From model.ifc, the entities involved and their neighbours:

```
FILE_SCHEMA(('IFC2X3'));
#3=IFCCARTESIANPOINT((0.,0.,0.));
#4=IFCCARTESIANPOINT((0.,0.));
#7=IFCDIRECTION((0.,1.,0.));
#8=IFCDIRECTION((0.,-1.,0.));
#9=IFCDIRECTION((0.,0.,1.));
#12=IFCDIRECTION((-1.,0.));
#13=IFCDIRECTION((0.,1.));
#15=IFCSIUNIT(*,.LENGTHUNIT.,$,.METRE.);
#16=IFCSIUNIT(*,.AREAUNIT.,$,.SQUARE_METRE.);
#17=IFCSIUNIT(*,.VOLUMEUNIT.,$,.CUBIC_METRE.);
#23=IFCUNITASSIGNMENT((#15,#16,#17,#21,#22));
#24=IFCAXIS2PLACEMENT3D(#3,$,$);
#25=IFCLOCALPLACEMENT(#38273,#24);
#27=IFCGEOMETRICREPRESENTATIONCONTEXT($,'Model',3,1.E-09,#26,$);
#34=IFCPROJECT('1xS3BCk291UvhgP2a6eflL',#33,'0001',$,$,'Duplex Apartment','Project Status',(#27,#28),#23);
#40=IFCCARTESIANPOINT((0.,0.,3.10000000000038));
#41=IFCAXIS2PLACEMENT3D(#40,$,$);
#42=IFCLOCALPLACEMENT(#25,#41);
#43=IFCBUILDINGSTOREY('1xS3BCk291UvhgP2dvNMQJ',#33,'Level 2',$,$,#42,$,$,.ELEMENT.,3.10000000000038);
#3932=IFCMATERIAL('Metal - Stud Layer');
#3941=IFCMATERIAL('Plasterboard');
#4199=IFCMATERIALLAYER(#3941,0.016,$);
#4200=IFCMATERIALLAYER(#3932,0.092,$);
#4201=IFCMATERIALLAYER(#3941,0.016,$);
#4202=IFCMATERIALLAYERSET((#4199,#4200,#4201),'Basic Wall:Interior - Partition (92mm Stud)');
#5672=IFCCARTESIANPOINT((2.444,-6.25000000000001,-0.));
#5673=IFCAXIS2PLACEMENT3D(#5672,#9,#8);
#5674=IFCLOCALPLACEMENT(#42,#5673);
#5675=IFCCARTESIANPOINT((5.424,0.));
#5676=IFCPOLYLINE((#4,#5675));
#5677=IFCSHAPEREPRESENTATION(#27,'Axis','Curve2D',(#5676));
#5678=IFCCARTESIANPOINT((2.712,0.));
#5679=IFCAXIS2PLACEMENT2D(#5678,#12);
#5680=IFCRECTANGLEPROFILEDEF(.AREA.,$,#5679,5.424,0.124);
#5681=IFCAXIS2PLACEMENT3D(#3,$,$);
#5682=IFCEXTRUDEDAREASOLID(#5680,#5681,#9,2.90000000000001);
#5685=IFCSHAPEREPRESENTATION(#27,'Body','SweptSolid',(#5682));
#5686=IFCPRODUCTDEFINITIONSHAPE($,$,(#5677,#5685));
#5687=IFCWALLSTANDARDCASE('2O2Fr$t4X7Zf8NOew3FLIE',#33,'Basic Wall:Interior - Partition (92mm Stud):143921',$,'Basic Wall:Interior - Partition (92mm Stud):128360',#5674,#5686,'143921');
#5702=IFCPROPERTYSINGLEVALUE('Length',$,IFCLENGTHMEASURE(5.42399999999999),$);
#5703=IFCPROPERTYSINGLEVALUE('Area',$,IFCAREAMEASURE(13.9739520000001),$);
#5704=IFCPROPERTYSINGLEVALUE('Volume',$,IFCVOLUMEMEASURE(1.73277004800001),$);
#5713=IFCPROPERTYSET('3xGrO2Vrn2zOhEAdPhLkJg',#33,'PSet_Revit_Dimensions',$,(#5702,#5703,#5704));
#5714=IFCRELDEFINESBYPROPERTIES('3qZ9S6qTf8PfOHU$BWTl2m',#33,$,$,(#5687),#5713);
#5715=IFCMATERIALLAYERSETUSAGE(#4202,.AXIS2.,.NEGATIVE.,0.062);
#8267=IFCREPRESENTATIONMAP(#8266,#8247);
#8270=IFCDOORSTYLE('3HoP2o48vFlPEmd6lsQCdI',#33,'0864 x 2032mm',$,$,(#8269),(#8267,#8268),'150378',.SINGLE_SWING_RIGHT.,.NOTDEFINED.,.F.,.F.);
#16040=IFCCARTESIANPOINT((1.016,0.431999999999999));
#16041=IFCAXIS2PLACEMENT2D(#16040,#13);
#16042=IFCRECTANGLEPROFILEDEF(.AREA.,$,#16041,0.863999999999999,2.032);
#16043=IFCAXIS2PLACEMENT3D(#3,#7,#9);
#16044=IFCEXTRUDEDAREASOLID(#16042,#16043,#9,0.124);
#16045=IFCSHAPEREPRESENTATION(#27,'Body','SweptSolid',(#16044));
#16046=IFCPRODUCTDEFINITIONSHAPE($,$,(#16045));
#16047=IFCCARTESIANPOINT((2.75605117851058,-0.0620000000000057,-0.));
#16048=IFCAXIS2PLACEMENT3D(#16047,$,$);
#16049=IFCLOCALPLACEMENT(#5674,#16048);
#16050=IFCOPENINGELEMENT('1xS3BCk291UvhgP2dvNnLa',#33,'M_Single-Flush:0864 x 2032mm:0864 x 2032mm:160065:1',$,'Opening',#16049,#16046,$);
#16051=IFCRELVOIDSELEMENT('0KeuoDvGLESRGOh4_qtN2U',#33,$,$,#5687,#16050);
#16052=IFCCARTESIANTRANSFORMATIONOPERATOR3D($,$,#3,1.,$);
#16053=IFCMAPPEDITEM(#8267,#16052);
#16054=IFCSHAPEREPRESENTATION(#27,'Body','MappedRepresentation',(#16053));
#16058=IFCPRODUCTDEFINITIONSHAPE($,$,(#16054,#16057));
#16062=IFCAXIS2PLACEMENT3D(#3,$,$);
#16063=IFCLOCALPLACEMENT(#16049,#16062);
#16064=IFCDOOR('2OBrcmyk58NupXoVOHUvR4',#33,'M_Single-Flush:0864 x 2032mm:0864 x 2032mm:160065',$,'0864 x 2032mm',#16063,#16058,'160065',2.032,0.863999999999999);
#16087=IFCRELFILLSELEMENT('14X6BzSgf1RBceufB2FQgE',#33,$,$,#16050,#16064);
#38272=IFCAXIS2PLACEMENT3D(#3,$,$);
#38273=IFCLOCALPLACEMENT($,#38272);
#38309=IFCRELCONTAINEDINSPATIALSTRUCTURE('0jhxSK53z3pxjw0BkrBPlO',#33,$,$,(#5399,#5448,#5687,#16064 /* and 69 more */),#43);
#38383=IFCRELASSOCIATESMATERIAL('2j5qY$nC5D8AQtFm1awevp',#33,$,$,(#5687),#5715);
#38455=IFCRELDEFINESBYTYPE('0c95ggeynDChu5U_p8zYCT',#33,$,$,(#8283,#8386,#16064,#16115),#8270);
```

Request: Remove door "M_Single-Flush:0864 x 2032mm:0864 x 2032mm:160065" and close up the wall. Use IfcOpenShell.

```python
import ifcopenshell
import ifcopenshell.api.feature
import ifcopenshell.api.pset
import ifcopenshell.api.root
import ifcopenshell.geom
import ifcopenshell.util.element
import ifcopenshell.util.shape
import ifcopenshell.util.unit

model = ifcopenshell.open("model.ifc")
area_scale = ifcopenshell.util.unit.calculate_unit_scale(model, "AREAUNIT")
volume_scale = ifcopenshell.util.unit.calculate_unit_scale(model, "VOLUMEUNIT")
settings = ifcopenshell.geom.settings()


def volume(element):
    """Net volume in cubic metres, openings subtracted."""
    shape = ifcopenshell.geom.create_shape(settings, element)
    return ifcopenshell.util.shape.get_volume(shape.geometry)


door = model.by_guid("2OBrcmyk58NupXoVOHUvR4")
opening = door.FillsVoids[0].RelatingOpeningElement
wall = opening.VoidsElements[0].RelatingBuildingElement
before = volume(wall)

ifcopenshell.api.root.remove_product(model, product=door)
ifcopenshell.api.feature.remove_feature(model, feature=opening)

after = volume(wall)
thickness = 0.124  # wall thickness in metres

# Update the wall's stored quantities.
pset = model.by_id(ifcopenshell.util.element.get_pset(wall, "PSet_Revit_Dimensions", should_inherit=False)["id"])
ifcopenshell.api.pset.edit_pset(model, pset=pset, properties={
    "Area": model.create_entity("IfcAreaMeasure", after / thickness / area_scale),
    "Volume": model.create_entity("IfcVolumeMeasure", after / volume_scale),
})

print(f"wall volume {before:.3f} -> {after:.3f} m3")

model.write("model-out.ifc")
```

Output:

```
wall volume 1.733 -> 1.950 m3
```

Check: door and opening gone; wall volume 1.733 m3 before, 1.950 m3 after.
